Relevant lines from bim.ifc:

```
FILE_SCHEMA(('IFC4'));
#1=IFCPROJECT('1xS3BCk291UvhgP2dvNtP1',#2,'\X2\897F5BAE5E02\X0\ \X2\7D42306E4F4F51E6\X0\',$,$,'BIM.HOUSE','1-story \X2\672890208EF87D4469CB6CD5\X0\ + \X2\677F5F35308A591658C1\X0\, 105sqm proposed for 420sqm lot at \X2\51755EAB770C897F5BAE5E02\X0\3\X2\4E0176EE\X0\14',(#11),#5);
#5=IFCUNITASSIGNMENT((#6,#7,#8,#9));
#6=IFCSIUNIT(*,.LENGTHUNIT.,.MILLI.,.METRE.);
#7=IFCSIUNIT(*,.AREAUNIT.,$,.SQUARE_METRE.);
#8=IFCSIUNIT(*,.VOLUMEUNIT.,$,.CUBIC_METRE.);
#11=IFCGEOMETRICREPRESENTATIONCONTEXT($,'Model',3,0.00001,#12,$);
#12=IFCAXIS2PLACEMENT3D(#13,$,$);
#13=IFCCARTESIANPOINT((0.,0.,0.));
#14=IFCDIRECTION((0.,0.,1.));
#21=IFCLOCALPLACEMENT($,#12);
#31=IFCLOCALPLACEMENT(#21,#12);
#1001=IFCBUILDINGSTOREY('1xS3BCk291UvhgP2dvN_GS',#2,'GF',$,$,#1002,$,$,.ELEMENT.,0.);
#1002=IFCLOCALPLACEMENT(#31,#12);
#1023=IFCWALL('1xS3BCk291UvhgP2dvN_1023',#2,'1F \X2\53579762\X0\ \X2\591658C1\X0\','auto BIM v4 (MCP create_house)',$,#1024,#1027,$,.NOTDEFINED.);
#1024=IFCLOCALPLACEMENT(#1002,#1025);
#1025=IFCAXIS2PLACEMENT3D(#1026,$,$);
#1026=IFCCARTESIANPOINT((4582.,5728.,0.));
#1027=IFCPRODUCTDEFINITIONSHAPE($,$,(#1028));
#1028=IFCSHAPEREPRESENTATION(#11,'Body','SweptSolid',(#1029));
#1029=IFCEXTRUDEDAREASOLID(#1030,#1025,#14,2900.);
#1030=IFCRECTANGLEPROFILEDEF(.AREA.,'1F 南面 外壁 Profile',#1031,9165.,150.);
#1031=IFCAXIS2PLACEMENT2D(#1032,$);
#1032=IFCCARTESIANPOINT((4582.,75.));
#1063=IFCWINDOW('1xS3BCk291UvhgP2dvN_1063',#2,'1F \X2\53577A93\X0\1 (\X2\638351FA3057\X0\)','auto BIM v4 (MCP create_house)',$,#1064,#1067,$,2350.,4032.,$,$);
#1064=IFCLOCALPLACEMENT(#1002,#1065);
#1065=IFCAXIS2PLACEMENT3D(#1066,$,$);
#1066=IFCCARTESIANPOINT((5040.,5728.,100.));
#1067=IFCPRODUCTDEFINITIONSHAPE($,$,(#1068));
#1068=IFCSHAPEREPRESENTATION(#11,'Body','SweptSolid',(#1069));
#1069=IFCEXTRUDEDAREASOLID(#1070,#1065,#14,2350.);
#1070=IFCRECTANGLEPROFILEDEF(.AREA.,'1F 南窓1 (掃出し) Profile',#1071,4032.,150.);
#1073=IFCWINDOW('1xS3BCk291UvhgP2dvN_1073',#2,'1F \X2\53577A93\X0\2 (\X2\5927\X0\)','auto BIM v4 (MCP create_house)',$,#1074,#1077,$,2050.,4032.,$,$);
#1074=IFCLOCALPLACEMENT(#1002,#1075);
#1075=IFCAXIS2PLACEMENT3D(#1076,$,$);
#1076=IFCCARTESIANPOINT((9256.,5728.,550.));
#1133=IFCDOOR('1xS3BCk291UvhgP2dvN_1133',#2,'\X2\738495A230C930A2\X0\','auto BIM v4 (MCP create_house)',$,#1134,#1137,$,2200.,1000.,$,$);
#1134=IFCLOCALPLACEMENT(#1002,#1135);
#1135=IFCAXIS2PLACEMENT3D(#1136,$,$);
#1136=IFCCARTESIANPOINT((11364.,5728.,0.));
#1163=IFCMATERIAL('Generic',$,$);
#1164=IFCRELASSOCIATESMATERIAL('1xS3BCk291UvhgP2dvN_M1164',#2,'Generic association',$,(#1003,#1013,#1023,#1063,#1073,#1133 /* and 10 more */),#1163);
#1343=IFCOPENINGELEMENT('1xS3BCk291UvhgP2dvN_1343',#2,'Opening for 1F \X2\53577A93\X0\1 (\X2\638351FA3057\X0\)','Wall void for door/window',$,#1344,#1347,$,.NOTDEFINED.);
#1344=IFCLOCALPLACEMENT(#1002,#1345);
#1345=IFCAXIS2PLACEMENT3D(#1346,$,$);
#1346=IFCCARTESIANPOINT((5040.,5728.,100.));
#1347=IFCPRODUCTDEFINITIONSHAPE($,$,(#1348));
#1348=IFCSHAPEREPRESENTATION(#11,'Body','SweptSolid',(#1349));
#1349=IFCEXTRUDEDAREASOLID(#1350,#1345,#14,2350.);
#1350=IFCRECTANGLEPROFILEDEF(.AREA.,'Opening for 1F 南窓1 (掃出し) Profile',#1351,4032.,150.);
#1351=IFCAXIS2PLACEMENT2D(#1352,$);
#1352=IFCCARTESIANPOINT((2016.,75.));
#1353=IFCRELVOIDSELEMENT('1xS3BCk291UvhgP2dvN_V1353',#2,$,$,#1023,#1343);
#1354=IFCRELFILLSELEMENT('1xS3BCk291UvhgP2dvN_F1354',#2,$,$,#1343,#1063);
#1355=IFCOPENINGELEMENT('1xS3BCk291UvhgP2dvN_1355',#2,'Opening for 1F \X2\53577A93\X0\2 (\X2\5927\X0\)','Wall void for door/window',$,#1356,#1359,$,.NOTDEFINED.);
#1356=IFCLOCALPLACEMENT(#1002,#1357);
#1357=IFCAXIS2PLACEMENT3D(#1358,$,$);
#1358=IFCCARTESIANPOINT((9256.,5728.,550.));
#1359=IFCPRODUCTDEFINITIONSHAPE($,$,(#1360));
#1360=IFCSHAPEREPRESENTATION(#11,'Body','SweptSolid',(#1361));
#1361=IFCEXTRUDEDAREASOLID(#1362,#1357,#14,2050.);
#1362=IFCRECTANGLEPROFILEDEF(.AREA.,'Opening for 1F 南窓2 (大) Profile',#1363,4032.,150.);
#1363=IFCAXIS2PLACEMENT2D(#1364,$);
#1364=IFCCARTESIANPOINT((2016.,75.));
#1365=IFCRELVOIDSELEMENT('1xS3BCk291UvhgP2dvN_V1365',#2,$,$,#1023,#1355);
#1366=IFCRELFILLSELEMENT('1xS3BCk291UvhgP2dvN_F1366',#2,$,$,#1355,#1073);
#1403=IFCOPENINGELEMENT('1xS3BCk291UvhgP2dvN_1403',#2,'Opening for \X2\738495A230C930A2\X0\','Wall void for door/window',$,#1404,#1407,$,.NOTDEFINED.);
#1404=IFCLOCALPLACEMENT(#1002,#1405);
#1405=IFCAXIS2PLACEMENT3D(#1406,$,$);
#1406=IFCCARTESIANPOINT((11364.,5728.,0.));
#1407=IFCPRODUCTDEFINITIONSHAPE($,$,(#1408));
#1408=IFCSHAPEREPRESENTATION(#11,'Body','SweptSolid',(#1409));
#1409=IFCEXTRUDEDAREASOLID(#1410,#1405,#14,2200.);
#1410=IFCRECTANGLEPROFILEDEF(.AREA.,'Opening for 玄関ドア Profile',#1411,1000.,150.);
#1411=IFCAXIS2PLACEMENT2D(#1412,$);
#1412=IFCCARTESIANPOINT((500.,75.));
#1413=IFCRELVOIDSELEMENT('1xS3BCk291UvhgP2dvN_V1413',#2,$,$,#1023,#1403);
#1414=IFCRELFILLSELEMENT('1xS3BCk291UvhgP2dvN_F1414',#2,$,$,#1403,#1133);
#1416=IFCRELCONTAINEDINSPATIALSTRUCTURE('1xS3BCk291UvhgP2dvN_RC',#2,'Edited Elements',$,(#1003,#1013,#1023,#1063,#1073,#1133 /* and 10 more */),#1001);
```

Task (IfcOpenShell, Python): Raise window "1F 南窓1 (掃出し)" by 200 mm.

```python
import numpy as np
import ifcopenshell
import ifcopenshell.api.geometry
import ifcopenshell.util.placement
import ifcopenshell.util.unit

model = ifcopenshell.open("bim.ifc")
unit_scale = ifcopenshell.util.unit.calculate_unit_scale(model)

window = model.by_guid("1xS3BCk291UvhgP2dvN_1063")
opening = window.FillsVoids[0].RelatingOpeningElement
dz = 200.0

shift = np.array([0.0, 0.0, dz])
# The window is not placed relative to its opening, so move both.
for product in (opening, window):
    matrix = ifcopenshell.util.placement.get_local_placement(product.ObjectPlacement)
    matrix[:3, 3] += shift
    ifcopenshell.api.geometry.edit_object_placement(model, product=product, matrix=matrix, is_si=False)

print(f"moved by {dz * unit_scale:+.3f} m")

model.write("bim-out.ifc")
```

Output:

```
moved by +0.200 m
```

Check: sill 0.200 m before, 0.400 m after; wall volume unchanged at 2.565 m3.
